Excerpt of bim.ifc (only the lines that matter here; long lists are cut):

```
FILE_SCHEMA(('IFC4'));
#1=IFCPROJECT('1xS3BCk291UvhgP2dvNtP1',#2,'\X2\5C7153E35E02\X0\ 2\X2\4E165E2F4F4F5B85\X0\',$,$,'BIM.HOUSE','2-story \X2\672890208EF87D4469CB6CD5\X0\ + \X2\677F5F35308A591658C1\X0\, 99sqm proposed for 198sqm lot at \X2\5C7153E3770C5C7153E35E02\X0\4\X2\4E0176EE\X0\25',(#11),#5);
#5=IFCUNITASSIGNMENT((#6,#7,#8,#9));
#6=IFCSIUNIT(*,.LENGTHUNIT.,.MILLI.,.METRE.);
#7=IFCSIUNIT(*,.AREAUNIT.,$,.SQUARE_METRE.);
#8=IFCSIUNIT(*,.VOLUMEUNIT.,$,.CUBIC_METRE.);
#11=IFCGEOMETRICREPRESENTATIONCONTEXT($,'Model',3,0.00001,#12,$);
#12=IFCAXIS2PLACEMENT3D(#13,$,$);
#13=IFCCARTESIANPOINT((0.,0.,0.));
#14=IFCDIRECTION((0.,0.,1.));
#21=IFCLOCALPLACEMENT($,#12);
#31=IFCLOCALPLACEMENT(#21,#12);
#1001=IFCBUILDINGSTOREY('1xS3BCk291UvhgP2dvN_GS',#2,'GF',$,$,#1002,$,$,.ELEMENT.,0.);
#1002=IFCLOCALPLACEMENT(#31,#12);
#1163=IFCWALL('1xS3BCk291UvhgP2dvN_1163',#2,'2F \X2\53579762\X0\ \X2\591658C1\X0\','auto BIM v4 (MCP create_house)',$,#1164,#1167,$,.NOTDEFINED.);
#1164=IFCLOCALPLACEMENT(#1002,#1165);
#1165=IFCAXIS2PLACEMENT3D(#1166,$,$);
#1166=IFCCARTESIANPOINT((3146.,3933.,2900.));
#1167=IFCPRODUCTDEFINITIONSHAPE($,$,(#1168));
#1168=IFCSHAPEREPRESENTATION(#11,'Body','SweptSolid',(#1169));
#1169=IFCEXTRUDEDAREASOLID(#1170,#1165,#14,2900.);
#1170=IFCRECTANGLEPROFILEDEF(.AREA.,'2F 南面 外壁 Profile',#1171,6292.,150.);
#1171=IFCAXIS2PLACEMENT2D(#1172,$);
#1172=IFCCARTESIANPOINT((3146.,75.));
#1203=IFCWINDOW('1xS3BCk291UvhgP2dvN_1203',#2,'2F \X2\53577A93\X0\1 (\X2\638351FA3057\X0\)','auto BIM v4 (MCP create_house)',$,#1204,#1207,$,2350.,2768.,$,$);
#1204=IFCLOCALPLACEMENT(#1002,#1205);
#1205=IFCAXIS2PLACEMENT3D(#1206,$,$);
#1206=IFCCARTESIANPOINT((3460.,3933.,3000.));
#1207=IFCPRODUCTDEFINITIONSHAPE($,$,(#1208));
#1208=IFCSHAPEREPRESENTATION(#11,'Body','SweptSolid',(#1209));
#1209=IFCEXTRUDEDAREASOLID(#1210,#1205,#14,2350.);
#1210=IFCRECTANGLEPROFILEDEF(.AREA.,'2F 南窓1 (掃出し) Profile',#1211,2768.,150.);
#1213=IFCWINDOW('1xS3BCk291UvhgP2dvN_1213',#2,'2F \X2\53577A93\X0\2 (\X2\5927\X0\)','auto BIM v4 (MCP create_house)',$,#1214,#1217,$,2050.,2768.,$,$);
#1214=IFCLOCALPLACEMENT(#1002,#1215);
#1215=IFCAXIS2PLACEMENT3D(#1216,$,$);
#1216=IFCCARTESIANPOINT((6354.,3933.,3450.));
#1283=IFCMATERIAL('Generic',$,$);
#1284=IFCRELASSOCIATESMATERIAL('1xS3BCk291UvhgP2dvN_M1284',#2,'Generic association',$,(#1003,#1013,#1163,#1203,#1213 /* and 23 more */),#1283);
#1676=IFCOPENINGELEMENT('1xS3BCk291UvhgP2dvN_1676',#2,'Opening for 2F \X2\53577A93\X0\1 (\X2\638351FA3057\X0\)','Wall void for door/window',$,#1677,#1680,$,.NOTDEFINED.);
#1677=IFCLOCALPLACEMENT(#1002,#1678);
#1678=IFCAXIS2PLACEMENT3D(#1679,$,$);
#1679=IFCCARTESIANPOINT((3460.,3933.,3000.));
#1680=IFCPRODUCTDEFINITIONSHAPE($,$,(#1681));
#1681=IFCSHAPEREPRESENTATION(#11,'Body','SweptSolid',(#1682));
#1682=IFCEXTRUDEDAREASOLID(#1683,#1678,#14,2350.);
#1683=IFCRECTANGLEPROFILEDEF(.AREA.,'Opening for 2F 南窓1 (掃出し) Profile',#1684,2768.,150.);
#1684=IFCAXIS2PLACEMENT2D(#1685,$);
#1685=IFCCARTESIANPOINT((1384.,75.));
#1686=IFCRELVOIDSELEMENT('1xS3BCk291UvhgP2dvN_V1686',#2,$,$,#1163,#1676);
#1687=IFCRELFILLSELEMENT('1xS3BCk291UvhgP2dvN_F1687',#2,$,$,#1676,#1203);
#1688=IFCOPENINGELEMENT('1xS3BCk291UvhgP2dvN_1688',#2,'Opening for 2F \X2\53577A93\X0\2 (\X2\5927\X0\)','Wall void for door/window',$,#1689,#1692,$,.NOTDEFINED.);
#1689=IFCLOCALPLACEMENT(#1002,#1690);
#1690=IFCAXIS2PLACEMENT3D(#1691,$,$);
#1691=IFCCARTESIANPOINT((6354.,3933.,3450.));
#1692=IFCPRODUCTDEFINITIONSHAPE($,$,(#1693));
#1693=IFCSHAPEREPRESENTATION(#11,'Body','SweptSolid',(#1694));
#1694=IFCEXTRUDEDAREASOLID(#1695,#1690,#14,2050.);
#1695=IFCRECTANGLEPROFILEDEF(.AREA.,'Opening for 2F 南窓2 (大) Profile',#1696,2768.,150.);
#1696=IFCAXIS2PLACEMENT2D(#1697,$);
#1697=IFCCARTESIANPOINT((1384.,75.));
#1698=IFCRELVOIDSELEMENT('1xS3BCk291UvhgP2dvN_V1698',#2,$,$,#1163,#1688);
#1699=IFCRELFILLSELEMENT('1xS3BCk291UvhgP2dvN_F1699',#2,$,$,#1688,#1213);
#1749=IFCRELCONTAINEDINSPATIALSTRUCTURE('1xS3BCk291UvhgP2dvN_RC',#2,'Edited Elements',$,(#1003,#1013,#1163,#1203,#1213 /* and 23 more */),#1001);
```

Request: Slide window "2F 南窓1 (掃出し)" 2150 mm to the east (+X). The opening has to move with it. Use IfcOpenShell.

```python
import ifcopenshell
import ifcopenshell.api.geometry
import ifcopenshell.util.placement
import ifcopenshell.util.unit

model = ifcopenshell.open("bim.ifc")
unit_scale = ifcopenshell.util.unit.calculate_unit_scale(model)

window = model.by_id(1203)
opening = window.FillsVoids[0].RelatingOpeningElement
wall = opening.VoidsElements[0].RelatingBuildingElement

wall_matrix = ifcopenshell.util.placement.get_local_placement(wall.ObjectPlacement)
shift = wall_matrix[:3, 0] * 2.15 / unit_scale
before = ifcopenshell.util.placement.get_local_placement(window.ObjectPlacement)[:3, 3].copy()

# The window is not placed relative to its opening, so move both.
for product in (opening, window):
    matrix = ifcopenshell.util.placement.get_local_placement(product.ObjectPlacement)
    matrix[:3, 3] += shift
    ifcopenshell.api.geometry.edit_object_placement(model, product=product, matrix=matrix, is_si=False)

after = ifcopenshell.util.placement.get_local_placement(window.ObjectPlacement)[:3, 3]
print("window moved by", (after - before).round(3) + 0.0)

model.write("bim_v2.ifc")
```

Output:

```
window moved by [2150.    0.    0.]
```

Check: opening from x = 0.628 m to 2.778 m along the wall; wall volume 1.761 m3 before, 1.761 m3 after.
